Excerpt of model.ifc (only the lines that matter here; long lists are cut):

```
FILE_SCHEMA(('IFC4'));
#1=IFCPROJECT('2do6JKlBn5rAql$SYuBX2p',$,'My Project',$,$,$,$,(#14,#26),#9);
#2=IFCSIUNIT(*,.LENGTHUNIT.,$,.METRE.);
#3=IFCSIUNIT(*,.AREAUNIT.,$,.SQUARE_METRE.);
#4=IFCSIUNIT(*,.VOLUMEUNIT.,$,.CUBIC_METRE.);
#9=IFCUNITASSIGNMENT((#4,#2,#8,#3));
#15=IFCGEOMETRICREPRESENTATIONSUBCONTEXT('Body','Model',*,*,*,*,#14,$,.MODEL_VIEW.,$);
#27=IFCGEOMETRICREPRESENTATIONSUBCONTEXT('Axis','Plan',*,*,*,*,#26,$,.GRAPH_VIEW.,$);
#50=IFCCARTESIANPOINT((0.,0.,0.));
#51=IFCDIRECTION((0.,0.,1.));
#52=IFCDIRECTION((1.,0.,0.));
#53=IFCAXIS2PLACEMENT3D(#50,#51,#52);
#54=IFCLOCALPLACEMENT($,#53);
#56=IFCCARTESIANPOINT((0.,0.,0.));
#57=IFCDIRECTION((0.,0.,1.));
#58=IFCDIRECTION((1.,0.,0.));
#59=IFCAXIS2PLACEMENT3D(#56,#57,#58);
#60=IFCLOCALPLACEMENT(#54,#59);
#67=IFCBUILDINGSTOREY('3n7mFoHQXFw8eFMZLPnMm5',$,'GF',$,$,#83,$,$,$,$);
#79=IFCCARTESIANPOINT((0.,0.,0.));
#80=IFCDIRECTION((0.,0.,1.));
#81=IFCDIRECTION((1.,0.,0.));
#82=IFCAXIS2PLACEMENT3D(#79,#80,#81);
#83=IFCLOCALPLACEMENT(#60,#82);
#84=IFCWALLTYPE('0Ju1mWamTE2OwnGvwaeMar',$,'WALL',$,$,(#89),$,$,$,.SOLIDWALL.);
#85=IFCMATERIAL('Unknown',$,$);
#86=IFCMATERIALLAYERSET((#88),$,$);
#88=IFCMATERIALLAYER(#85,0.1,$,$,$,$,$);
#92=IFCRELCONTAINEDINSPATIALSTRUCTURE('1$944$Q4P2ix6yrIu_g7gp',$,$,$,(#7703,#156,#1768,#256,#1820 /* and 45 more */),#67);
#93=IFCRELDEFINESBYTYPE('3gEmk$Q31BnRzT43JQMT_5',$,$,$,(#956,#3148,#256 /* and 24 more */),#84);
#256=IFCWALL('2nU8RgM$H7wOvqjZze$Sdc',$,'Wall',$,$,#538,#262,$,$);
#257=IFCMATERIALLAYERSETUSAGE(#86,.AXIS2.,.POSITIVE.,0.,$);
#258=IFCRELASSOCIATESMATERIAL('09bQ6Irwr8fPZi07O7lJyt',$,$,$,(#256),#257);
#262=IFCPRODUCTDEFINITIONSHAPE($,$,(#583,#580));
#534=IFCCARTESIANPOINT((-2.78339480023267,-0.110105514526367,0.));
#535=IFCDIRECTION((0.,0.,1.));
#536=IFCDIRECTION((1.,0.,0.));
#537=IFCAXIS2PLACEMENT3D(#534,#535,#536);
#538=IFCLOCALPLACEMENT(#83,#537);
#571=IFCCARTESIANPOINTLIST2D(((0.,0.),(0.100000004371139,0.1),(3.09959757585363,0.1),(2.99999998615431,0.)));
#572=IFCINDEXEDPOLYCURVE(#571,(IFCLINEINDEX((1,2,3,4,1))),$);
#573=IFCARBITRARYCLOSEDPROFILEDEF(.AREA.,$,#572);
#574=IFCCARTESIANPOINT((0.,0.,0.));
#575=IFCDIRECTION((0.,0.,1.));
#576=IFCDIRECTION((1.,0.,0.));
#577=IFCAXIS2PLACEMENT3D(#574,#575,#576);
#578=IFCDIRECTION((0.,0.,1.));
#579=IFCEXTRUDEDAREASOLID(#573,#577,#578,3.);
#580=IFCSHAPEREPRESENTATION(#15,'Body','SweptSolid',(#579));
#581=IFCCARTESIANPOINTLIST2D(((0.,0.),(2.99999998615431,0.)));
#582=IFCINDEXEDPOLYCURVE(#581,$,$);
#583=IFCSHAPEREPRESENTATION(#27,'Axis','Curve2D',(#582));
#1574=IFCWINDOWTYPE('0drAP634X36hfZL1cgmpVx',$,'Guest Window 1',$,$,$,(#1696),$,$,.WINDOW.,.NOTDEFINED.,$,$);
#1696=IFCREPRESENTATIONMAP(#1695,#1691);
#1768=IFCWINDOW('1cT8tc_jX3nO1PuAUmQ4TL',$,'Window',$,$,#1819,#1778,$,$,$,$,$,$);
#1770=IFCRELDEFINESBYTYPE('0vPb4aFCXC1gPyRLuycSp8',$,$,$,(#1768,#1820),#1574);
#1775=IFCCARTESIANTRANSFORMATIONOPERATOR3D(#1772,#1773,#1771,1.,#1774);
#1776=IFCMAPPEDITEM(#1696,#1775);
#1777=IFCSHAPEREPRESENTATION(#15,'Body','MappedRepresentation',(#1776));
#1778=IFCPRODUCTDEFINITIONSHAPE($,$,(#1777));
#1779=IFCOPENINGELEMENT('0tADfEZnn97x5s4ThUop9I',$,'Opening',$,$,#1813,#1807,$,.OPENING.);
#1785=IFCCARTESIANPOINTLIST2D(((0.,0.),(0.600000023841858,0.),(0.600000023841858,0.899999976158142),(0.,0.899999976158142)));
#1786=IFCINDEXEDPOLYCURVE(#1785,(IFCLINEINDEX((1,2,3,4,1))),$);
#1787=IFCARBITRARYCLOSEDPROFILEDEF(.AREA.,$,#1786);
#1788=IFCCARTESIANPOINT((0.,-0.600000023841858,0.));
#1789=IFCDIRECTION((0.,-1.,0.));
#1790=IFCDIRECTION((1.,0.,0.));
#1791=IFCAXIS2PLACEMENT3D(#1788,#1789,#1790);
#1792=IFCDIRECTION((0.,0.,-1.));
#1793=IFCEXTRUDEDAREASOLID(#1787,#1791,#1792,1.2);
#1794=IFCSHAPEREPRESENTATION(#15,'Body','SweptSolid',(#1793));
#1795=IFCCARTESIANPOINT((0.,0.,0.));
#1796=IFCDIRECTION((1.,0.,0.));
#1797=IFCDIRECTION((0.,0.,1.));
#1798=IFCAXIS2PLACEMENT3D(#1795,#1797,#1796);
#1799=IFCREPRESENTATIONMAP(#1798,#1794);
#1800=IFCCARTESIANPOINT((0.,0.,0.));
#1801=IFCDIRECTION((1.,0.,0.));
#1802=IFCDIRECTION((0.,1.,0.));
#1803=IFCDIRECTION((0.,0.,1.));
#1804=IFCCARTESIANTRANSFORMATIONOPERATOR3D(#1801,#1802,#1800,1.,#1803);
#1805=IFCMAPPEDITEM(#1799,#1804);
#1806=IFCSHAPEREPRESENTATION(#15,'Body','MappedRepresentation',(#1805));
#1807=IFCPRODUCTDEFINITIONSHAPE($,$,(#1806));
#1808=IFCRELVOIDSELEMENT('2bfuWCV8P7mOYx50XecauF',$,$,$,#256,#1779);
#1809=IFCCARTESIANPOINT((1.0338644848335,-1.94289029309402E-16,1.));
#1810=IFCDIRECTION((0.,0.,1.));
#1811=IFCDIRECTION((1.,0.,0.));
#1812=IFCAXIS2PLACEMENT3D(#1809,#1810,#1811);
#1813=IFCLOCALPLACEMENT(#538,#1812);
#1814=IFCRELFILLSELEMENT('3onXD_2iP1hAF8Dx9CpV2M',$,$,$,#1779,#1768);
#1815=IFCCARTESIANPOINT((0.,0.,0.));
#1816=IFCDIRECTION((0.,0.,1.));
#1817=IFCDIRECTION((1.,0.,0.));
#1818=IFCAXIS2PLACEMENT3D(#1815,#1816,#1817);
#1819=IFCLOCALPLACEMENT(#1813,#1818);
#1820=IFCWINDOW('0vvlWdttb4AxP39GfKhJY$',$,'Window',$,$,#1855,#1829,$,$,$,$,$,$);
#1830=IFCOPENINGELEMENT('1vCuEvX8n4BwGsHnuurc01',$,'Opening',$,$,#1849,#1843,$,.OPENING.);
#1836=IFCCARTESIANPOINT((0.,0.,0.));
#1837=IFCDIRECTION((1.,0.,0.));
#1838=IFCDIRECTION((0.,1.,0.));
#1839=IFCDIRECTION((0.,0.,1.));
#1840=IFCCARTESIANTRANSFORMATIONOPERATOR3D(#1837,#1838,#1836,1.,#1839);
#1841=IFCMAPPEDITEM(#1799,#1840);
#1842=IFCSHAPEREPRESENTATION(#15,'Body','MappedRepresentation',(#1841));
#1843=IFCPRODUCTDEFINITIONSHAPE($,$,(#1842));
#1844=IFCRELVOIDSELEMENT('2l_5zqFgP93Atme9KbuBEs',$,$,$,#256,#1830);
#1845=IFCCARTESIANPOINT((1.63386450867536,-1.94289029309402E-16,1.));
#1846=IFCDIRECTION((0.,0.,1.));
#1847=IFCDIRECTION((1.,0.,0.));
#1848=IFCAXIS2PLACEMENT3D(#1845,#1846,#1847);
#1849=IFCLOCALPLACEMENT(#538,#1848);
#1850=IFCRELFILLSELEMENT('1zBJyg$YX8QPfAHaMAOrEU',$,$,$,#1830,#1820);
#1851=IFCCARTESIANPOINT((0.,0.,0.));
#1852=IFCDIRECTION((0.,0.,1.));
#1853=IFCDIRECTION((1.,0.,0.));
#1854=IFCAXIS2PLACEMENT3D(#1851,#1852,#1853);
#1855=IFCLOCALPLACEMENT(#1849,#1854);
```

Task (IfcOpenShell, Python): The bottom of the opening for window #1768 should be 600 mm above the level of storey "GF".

```python
import numpy as np
import ifcopenshell
import ifcopenshell.api.geometry
import ifcopenshell.geom
import ifcopenshell.util.element
import ifcopenshell.util.placement
import ifcopenshell.util.shape
import ifcopenshell.util.unit

model = ifcopenshell.open("model.ifc")
unit_scale = ifcopenshell.util.unit.calculate_unit_scale(model)

window = model.by_guid("1cT8tc_jX3nO1PuAUmQ4TL")
opening = window.FillsVoids[0].RelatingOpeningElement
storey = ifcopenshell.util.element.get_container(window, ifc_class="IfcBuildingStorey")
level = ifcopenshell.util.placement.get_local_placement(storey.ObjectPlacement)[2, 3]

# The opening's origin need not be at the sill, so measure its lowest point.
shape = ifcopenshell.geom.create_shape(ifcopenshell.geom.settings(), opening)
bottom = ifcopenshell.util.shape.get_shape_bottom_elevation(shape, shape.geometry) / unit_scale
dz = level + 0.6 / unit_scale - bottom

shift = np.array([0.0, 0.0, dz])
# The window is placed relative to its opening, so it follows when the opening moves.
matrix = ifcopenshell.util.placement.get_local_placement(opening.ObjectPlacement)
matrix[:3, 3] += shift
ifcopenshell.api.geometry.edit_object_placement(
    model, product=opening, matrix=matrix, is_si=False, should_transform_children=True
)

print(f"moved by {dz * unit_scale:+.3f} m")

model.write("model-out.ifc")
```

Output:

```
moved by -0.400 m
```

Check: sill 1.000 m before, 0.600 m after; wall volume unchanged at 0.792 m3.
